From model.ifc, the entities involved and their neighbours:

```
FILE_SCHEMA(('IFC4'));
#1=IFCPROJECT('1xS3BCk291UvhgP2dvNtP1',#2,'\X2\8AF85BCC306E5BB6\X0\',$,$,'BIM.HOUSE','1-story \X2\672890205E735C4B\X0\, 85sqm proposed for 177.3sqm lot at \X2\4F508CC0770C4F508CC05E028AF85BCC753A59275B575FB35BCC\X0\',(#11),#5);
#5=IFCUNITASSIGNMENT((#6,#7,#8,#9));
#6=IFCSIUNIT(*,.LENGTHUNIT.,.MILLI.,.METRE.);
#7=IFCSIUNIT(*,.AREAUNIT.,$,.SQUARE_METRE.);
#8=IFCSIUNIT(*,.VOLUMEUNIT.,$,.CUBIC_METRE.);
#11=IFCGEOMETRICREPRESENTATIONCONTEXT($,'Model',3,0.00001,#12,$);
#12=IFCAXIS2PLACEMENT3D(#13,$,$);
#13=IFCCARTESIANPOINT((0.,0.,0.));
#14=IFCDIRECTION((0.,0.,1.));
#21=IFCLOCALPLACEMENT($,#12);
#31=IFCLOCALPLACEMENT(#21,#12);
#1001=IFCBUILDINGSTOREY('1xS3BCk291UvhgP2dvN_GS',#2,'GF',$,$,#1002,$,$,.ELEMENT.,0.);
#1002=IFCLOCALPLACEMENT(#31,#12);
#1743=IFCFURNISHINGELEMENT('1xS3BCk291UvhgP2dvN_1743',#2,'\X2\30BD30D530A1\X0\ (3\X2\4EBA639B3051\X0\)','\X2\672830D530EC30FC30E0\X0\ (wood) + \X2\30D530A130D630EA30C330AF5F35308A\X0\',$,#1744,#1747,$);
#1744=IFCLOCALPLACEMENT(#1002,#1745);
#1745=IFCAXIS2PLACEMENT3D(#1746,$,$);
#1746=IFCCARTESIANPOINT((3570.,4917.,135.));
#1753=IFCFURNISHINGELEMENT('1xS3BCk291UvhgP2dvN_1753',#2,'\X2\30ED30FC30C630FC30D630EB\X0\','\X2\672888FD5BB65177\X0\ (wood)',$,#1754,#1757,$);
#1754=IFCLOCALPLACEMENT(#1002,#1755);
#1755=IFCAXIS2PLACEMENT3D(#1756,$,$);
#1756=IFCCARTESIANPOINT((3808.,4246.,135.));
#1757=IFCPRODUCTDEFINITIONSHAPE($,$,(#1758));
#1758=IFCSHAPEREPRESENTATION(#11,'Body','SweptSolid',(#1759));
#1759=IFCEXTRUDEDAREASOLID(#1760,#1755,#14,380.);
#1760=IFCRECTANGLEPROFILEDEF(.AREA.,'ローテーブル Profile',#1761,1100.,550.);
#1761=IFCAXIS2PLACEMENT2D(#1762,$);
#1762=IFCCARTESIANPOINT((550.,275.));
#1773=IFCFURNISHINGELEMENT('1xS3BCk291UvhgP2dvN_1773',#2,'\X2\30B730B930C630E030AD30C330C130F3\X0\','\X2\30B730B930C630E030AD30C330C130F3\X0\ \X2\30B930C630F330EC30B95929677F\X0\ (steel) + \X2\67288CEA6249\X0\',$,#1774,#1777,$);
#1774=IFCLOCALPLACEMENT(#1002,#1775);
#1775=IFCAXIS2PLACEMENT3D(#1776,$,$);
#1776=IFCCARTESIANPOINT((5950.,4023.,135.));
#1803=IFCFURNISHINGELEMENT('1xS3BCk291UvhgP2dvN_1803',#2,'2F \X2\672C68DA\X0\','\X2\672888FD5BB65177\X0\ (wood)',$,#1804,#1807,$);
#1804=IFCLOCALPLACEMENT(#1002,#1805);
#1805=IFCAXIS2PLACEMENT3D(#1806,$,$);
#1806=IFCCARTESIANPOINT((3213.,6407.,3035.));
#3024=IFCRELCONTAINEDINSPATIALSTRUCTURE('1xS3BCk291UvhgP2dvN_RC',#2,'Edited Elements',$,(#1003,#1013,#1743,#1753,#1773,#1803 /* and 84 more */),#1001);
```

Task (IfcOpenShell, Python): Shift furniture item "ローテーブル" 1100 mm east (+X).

```python
import ifcopenshell
import ifcopenshell.api.geometry
import ifcopenshell.util.placement

model = ifcopenshell.open("model.ifc")

item = model.by_id(1753)
matrix = ifcopenshell.util.placement.get_local_placement(item.ObjectPlacement)
matrix[0, 3] += 1100.0
ifcopenshell.api.geometry.edit_object_placement(model, product=item, matrix=matrix, is_si=False)

print(ifcopenshell.util.placement.get_local_placement(item.ObjectPlacement).round(3) + 0.0)

model.write("model_edited.ifc")
```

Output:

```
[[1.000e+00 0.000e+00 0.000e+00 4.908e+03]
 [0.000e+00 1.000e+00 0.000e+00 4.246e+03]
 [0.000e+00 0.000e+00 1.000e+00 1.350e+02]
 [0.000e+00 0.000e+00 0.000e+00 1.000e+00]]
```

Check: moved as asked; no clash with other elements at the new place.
